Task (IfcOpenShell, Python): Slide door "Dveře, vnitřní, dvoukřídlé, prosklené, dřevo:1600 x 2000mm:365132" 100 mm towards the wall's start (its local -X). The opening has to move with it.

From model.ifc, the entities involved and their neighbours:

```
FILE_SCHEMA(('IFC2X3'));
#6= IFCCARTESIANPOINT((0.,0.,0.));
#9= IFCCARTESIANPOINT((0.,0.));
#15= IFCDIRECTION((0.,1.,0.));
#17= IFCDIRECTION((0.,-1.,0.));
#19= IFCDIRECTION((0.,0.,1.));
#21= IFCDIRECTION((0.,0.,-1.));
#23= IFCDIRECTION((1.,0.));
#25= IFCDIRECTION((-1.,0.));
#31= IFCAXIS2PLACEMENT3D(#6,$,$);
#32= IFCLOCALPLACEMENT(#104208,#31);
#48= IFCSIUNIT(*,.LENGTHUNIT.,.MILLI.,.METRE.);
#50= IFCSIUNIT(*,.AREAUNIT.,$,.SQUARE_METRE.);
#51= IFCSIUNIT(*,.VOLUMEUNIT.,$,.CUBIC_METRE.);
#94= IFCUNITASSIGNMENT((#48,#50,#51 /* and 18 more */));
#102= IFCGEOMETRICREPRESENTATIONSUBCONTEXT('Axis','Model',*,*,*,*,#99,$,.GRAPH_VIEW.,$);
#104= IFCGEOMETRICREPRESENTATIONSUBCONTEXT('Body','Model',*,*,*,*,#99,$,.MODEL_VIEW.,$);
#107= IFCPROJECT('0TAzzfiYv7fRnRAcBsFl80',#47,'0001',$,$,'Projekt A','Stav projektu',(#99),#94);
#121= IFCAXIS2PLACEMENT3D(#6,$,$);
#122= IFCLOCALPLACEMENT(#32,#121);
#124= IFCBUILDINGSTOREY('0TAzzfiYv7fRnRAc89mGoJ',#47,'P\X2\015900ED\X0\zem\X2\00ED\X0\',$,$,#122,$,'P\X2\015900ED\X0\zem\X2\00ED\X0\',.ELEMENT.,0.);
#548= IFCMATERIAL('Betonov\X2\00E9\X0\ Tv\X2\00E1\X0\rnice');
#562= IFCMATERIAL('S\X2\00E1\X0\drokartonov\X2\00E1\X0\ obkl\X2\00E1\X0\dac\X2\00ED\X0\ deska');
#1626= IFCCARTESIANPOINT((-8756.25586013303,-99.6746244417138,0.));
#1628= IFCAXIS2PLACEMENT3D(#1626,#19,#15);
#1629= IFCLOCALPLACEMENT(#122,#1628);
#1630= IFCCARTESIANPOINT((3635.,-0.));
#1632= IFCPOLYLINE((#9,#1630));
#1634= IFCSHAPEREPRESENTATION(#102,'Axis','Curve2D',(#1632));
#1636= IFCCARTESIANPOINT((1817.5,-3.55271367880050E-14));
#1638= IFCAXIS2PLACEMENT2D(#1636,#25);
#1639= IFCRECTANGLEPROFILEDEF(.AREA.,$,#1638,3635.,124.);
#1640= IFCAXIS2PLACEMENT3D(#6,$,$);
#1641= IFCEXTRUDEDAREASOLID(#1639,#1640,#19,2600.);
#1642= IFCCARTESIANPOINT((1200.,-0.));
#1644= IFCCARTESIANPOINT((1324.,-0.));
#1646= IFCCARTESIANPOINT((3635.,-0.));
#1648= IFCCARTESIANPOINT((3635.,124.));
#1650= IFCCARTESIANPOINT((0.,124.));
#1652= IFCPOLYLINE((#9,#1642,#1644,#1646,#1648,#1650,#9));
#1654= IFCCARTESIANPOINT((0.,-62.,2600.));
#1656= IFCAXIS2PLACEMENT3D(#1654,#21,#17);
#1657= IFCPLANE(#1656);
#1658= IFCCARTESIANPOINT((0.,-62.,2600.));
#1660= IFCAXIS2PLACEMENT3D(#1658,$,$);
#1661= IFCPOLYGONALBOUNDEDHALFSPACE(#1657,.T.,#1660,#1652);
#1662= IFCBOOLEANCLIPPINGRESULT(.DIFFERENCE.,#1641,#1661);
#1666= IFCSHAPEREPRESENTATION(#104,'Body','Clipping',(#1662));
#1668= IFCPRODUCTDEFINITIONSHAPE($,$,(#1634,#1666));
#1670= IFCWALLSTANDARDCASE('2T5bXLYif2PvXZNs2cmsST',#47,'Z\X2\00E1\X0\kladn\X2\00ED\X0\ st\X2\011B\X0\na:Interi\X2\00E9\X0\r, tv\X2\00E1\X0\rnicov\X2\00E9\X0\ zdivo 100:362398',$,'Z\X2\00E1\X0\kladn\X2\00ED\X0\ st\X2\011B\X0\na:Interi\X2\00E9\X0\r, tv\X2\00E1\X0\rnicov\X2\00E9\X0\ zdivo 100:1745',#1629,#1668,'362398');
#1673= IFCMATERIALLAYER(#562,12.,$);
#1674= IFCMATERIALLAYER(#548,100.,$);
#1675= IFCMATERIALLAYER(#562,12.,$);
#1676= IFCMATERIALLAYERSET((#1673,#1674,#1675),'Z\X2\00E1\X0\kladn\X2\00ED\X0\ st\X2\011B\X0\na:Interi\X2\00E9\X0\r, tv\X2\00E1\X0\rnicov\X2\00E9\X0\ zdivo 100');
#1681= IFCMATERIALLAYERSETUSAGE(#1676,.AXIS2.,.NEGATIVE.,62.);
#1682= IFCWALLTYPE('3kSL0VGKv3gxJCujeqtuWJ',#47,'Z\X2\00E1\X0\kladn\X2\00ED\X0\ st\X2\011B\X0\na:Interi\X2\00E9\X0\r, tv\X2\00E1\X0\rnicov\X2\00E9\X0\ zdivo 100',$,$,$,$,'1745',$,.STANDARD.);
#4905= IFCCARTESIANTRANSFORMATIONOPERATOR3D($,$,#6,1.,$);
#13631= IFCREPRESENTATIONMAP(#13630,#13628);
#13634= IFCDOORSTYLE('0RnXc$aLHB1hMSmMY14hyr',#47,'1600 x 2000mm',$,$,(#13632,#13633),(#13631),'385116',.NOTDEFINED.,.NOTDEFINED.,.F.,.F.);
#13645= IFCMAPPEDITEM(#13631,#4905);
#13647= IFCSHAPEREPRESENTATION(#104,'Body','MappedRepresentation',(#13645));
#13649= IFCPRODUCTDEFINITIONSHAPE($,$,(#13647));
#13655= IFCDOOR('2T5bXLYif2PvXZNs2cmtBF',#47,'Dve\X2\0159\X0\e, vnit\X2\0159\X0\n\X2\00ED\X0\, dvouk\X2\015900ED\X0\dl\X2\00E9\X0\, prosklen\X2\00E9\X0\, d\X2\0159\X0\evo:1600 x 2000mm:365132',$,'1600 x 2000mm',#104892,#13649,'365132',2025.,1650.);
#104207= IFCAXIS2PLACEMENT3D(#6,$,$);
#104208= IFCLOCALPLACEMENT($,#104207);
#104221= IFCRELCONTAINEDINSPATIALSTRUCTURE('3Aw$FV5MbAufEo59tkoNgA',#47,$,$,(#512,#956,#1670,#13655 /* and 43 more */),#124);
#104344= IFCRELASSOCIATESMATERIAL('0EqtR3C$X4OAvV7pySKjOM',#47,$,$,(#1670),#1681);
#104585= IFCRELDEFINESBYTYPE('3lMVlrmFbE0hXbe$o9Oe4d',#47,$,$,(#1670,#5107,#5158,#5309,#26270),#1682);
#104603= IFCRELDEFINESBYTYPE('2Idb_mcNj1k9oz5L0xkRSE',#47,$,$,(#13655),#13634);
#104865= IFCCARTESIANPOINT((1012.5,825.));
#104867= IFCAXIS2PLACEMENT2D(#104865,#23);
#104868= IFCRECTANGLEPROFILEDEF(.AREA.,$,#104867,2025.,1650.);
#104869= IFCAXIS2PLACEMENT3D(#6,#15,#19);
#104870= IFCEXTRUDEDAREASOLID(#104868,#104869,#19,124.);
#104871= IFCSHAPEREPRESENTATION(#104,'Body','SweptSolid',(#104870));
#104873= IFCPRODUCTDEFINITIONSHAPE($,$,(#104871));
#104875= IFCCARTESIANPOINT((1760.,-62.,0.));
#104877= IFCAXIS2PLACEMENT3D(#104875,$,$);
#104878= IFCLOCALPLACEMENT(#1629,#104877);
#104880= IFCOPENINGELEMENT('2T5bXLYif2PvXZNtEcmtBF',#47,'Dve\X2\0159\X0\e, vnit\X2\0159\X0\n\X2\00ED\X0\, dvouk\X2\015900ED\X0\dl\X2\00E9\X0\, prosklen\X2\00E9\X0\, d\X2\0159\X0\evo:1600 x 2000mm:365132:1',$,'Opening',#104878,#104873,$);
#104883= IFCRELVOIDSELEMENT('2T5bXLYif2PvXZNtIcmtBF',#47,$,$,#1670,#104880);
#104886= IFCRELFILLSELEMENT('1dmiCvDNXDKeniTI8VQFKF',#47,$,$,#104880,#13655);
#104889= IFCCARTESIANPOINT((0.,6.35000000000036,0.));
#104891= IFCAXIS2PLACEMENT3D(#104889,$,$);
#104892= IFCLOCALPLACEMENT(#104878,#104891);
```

```python
import ifcopenshell
import ifcopenshell.api.geometry
import ifcopenshell.util.placement
import ifcopenshell.util.unit

model = ifcopenshell.open("model.ifc")
unit_scale = ifcopenshell.util.unit.calculate_unit_scale(model)

door = model.by_id(13655)
opening = door.FillsVoids[0].RelatingOpeningElement
wall = opening.VoidsElements[0].RelatingBuildingElement

wall_matrix = ifcopenshell.util.placement.get_local_placement(wall.ObjectPlacement)
shift = wall_matrix[:3, 0] * -0.1 / unit_scale
before = ifcopenshell.util.placement.get_local_placement(door.ObjectPlacement)[:3, 3].copy()

# The door is placed relative to its opening, so it follows when the opening moves.
matrix = ifcopenshell.util.placement.get_local_placement(opening.ObjectPlacement)
matrix[:3, 3] += shift
ifcopenshell.api.geometry.edit_object_placement(
    model, product=opening, matrix=matrix, is_si=False, should_transform_children=True
)

after = ifcopenshell.util.placement.get_local_placement(door.ObjectPlacement)[:3, 3]
print("door moved by", (after - before).round(3) + 0.0)

model.write("model_v2.ifc")
```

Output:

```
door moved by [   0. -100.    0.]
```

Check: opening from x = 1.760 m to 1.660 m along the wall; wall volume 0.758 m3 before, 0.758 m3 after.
